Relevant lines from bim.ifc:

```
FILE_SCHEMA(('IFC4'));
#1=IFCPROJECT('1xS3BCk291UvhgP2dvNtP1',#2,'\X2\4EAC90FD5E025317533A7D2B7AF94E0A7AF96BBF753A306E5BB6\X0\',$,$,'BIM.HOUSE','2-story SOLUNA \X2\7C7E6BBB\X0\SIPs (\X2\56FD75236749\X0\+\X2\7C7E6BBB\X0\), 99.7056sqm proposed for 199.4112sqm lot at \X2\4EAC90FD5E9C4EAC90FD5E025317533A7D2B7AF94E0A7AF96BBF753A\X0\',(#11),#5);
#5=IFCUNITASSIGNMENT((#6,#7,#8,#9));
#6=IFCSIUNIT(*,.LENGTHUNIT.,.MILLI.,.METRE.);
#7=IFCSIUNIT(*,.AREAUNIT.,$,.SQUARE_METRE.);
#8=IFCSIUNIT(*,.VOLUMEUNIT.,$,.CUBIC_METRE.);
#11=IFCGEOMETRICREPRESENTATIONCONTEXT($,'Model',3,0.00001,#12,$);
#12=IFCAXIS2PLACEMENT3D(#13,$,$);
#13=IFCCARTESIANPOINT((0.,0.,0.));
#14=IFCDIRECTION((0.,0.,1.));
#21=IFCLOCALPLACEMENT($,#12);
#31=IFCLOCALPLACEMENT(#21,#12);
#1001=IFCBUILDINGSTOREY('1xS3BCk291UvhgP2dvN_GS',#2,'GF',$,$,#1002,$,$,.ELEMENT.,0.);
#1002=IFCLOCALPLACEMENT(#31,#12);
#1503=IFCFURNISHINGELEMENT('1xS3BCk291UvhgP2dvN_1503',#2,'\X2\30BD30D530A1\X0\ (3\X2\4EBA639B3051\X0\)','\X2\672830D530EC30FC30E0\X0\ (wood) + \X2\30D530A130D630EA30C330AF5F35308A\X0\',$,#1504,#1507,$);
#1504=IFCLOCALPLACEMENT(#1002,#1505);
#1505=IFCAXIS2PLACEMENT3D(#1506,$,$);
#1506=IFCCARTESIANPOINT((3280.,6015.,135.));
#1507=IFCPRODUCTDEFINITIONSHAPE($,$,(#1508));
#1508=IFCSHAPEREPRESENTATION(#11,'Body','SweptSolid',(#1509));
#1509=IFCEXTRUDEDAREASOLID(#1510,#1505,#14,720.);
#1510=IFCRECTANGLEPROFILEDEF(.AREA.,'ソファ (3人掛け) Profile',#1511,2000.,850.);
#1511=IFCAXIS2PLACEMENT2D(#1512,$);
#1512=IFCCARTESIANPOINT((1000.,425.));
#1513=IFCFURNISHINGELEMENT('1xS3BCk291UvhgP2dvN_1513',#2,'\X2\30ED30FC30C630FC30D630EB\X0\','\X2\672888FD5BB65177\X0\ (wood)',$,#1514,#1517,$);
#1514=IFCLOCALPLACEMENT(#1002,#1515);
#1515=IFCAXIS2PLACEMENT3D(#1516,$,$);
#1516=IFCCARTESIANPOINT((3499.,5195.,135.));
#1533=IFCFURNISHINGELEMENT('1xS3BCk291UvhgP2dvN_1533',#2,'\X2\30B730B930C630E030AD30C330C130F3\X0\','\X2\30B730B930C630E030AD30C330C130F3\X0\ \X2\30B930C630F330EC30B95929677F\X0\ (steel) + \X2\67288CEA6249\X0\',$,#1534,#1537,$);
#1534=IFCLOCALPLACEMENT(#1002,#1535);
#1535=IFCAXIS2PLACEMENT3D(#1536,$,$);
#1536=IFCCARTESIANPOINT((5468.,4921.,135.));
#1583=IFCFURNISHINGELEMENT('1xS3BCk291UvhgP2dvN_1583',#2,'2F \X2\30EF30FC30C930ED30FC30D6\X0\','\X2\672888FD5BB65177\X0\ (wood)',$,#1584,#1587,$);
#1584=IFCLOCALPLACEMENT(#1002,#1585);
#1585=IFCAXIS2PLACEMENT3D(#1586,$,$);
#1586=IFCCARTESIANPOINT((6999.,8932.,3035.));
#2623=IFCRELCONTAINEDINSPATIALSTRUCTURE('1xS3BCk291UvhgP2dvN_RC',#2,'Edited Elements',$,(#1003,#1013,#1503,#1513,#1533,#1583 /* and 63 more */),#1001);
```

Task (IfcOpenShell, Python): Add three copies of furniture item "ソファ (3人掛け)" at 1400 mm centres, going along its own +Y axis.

```python
import ifcopenshell
import ifcopenshell.api.geometry
import ifcopenshell.api.root
import ifcopenshell.util.element
import ifcopenshell.util.placement

model = ifcopenshell.open("bim.ifc")


def reuse_history(source, copy):
    """copy_class also copies each property set's owner history, people and application; keep the originals."""
    for rel in copy.IsDefinedBy:
        if rel.is_a("IfcRelDefinesByProperties") and (history := rel.RelatingPropertyDefinition.OwnerHistory):
            rel.RelatingPropertyDefinition.OwnerHistory = source.OwnerHistory
            ifcopenshell.util.element.remove_deep2(model, history)


source = model.by_guid("1xS3BCk291UvhgP2dvN_1503")
base = ifcopenshell.util.placement.get_local_placement(source.ObjectPlacement)
step = base[:3, 1] * 1400.0

for i in range(1, 4):
    copy = ifcopenshell.api.root.copy_class(model, product=source)
    copy.Representation = ifcopenshell.util.element.copy_deep(
        model, source.Representation, exclude=["IfcGeometricRepresentationContext", "IfcRepresentationMap"]
    )
    reuse_history(source, copy)
    matrix = base.copy()
    matrix[:3, 3] += i * step
    print("added at", matrix[:3, 3].round(3) + 0.0)
    ifcopenshell.api.geometry.edit_object_placement(model, product=copy, matrix=matrix, is_si=False)

model.write("bim-out.ifc")
```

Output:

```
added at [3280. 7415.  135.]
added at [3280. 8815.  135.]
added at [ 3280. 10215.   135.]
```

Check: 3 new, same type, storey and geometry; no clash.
